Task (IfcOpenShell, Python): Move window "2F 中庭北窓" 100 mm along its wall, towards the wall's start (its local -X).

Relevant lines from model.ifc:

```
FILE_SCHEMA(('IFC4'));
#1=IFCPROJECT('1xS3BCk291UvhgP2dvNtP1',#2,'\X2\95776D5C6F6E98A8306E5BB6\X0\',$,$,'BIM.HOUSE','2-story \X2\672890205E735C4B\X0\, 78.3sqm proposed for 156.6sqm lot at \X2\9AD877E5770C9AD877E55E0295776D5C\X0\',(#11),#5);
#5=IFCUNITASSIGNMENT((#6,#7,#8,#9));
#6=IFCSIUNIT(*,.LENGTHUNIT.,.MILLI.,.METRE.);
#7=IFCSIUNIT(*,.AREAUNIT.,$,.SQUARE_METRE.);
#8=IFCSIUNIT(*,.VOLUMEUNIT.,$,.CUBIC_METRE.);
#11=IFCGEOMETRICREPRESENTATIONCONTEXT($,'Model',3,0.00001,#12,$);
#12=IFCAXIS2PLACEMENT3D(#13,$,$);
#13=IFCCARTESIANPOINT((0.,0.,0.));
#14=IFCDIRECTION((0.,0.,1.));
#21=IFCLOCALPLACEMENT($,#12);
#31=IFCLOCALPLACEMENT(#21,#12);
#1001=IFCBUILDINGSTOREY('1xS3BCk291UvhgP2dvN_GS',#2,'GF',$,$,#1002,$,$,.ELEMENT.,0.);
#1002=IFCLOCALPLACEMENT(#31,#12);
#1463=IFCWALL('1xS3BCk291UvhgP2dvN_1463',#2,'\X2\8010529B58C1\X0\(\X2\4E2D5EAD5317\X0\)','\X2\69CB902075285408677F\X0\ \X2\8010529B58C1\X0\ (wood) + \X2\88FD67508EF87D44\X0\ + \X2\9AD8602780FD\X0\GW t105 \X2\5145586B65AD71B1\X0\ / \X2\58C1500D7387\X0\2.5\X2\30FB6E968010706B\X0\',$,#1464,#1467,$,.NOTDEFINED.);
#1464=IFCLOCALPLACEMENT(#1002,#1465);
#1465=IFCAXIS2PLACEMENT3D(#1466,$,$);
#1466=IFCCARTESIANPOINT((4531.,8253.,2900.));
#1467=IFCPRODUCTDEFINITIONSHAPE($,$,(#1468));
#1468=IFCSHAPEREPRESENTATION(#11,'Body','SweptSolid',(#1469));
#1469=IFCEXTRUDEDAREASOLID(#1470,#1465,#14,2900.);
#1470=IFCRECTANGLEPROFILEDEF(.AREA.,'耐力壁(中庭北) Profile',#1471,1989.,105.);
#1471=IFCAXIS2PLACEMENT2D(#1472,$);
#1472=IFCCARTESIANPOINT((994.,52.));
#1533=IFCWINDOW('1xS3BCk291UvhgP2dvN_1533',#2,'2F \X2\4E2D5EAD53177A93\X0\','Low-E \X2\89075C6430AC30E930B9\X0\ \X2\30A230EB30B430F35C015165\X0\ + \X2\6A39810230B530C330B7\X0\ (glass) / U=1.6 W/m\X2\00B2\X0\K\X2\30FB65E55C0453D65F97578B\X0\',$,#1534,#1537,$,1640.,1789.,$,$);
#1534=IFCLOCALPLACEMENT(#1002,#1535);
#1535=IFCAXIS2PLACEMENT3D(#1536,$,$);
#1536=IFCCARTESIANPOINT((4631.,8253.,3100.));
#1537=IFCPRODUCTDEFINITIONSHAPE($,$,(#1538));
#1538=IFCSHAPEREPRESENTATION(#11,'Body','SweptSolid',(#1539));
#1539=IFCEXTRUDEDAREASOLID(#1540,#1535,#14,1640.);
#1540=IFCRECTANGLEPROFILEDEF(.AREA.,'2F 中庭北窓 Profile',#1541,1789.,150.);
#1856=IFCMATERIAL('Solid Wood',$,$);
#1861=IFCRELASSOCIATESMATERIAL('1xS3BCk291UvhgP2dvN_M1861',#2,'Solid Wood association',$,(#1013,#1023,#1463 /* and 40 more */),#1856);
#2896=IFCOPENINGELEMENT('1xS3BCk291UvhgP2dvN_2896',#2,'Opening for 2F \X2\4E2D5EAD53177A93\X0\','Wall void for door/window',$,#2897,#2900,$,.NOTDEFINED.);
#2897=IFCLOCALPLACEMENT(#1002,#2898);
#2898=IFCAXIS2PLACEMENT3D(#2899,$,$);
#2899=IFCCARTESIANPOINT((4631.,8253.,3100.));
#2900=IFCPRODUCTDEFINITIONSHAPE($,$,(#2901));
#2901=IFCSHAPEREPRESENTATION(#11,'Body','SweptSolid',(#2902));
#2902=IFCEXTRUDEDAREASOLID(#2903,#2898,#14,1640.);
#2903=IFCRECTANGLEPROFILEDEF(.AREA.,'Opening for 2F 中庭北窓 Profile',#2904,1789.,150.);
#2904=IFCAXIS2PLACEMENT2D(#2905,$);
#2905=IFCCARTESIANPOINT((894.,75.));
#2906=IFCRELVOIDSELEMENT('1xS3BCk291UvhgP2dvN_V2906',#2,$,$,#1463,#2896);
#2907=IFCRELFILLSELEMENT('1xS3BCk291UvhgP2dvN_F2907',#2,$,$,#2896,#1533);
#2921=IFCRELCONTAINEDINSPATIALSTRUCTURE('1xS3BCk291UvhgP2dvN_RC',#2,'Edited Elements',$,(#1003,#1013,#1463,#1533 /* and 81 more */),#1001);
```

```python
import ifcopenshell
import ifcopenshell.api.geometry
import ifcopenshell.util.placement

model = ifcopenshell.open("model.ifc")

window = model.by_guid("1xS3BCk291UvhgP2dvN_1533")
opening = window.FillsVoids[0].RelatingOpeningElement
wall = opening.VoidsElements[0].RelatingBuildingElement

wall_matrix = ifcopenshell.util.placement.get_local_placement(wall.ObjectPlacement)
shift = wall_matrix[:3, 0] * -100.0
before = ifcopenshell.util.placement.get_local_placement(window.ObjectPlacement)[:3, 3].copy()

# The window is not placed relative to its opening, so move both.
for product in (opening, window):
    matrix = ifcopenshell.util.placement.get_local_placement(product.ObjectPlacement)
    matrix[:3, 3] += shift
    ifcopenshell.api.geometry.edit_object_placement(model, product=product, matrix=matrix, is_si=False)

after = ifcopenshell.util.placement.get_local_placement(window.ObjectPlacement)[:3, 3]
print("window moved by", (after - before).round(3) + 0.0)

model.write("model_updated.ifc")
```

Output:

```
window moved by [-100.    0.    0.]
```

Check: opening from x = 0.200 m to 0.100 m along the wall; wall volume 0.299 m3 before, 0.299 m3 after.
